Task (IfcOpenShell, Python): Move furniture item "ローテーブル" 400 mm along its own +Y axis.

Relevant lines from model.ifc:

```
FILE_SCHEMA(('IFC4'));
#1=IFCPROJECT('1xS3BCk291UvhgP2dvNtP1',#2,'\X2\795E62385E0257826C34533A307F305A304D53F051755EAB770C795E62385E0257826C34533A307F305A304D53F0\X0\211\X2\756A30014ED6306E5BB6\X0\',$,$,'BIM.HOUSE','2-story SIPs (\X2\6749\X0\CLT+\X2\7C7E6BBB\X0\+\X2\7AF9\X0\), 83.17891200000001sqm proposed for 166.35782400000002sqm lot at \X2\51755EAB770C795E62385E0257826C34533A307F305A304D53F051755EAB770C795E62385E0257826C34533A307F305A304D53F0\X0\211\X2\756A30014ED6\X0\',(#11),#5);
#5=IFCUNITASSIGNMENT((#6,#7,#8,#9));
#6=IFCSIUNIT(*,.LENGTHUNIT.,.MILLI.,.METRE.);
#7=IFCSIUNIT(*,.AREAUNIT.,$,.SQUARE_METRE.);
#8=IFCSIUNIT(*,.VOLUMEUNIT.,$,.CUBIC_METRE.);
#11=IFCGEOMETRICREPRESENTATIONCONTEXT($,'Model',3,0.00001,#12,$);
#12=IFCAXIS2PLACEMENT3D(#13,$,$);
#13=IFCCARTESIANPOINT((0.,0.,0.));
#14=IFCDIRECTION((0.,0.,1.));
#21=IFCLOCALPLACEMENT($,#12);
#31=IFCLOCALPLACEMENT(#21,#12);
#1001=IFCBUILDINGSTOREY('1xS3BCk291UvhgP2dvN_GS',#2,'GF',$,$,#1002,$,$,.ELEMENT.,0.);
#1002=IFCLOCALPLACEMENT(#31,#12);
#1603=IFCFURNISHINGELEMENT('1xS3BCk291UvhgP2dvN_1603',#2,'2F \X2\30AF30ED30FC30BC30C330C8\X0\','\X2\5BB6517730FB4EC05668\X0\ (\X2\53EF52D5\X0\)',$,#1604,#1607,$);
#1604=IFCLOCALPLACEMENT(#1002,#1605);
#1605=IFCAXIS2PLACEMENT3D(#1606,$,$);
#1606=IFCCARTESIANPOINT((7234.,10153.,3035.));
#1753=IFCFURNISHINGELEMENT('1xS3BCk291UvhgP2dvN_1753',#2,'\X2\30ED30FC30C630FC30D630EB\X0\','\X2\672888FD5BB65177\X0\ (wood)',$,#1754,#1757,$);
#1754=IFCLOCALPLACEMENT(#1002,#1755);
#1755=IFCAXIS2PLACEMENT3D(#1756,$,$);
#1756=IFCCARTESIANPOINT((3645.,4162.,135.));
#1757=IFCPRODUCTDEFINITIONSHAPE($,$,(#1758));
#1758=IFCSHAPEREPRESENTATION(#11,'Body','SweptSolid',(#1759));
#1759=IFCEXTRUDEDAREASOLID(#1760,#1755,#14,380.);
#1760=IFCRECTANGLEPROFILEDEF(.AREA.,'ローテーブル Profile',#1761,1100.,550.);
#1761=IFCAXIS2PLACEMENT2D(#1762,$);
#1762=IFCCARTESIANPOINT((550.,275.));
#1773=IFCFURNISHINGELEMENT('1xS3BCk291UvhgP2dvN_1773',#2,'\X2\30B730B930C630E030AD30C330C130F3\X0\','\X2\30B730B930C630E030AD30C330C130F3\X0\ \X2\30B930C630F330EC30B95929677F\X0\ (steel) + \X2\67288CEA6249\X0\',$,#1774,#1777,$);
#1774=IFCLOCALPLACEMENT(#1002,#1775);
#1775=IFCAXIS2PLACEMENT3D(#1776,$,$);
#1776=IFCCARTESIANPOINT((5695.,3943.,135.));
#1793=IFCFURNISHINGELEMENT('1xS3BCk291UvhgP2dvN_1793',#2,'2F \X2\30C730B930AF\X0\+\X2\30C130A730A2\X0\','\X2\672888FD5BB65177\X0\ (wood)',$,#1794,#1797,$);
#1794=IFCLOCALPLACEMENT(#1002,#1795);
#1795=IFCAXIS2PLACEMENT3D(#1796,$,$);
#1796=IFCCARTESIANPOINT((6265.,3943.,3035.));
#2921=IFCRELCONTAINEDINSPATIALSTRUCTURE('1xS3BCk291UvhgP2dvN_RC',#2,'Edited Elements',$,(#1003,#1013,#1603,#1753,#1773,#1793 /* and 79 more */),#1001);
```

```python
import ifcopenshell
import ifcopenshell.api.geometry
import ifcopenshell.util.placement

model = ifcopenshell.open("model.ifc")

item = model.by_guid("1xS3BCk291UvhgP2dvN_1753")
matrix = ifcopenshell.util.placement.get_local_placement(item.ObjectPlacement)
matrix[:3, 3] += matrix[:3, 1] * 400.0
ifcopenshell.api.geometry.edit_object_placement(model, product=item, matrix=matrix, is_si=False)

print(ifcopenshell.util.placement.get_local_placement(item.ObjectPlacement).round(3) + 0.0)

model.write("model-out.ifc")
```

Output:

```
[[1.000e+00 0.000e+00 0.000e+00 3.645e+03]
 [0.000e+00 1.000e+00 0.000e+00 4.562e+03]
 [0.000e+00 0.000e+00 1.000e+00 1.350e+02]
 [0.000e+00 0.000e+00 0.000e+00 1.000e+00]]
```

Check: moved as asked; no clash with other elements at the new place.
